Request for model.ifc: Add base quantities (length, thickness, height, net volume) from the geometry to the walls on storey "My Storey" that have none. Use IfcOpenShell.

First a look at what the model holds.

```python
import ifcopenshell
import ifcopenshell.util.element
import ifcopenshell.util.unit

model = ifcopenshell.open("model.ifc")
print(model.schema)
for unit_type in ("LENGTHUNIT", "AREAUNIT", "VOLUMEUNIT"):
    print(unit_type, ifcopenshell.util.unit.calculate_unit_scale(model, unit_type))
storey = next(s for s in model.by_type("IfcBuildingStorey") if s.Name == "My Storey")
walls = [e for e in ifcopenshell.util.element.get_decomposition(storey) if e.is_a("IfcWall")]
for e in sorted(walls, key=lambda e: e.id()):
    print(e.id(), e.is_a(), e.Name, list(ifcopenshell.util.element.get_psets(e, qtos_only=True)), sep=" | ")
```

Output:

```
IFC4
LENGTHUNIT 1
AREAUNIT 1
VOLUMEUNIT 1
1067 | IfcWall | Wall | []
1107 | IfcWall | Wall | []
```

```python
import ifcopenshell
import ifcopenshell.api.pset
import ifcopenshell.geom
import ifcopenshell.util.element
import ifcopenshell.util.shape
import ifcopenshell.util.unit

model = ifcopenshell.open("model.ifc")
unit_scale = ifcopenshell.util.unit.calculate_unit_scale(model)
volume_scale = ifcopenshell.util.unit.calculate_unit_scale(model, "VOLUMEUNIT")
settings = ifcopenshell.geom.settings()

storey = next(s for s in model.by_type("IfcBuildingStorey") if s.Name == "My Storey")
walls = [e for e in ifcopenshell.util.element.get_decomposition(storey) if e.is_a("IfcWall")]

for e in sorted(walls, key=lambda e: e.id()):
    if ifcopenshell.util.element.get_psets(e, qtos_only=True, should_inherit=False):
        continue
    # Geometry comes back in metres, in the element's own axes.
    shape = ifcopenshell.geom.create_shape(settings, e)
    values = {
        "Length": ifcopenshell.util.shape.get_x(shape.geometry) / unit_scale,
        "Width": ifcopenshell.util.shape.get_y(shape.geometry) / unit_scale,
        "Height": ifcopenshell.util.shape.get_z(shape.geometry) / unit_scale,
        "NetVolume": ifcopenshell.util.shape.get_volume(shape.geometry) / volume_scale,
    }
    qto = ifcopenshell.api.pset.add_qto(model, product=e, name="Qto_WallBaseQuantities")
    ifcopenshell.api.pset.edit_qto(model, qto=qto, properties=values)
    print(e.id(), {k: round(v, 3) for k, v in values.items()})

model.write("model_edited.ifc")
```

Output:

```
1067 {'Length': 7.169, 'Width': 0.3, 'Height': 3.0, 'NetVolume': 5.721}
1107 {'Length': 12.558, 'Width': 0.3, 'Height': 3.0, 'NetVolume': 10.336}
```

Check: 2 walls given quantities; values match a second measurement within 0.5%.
